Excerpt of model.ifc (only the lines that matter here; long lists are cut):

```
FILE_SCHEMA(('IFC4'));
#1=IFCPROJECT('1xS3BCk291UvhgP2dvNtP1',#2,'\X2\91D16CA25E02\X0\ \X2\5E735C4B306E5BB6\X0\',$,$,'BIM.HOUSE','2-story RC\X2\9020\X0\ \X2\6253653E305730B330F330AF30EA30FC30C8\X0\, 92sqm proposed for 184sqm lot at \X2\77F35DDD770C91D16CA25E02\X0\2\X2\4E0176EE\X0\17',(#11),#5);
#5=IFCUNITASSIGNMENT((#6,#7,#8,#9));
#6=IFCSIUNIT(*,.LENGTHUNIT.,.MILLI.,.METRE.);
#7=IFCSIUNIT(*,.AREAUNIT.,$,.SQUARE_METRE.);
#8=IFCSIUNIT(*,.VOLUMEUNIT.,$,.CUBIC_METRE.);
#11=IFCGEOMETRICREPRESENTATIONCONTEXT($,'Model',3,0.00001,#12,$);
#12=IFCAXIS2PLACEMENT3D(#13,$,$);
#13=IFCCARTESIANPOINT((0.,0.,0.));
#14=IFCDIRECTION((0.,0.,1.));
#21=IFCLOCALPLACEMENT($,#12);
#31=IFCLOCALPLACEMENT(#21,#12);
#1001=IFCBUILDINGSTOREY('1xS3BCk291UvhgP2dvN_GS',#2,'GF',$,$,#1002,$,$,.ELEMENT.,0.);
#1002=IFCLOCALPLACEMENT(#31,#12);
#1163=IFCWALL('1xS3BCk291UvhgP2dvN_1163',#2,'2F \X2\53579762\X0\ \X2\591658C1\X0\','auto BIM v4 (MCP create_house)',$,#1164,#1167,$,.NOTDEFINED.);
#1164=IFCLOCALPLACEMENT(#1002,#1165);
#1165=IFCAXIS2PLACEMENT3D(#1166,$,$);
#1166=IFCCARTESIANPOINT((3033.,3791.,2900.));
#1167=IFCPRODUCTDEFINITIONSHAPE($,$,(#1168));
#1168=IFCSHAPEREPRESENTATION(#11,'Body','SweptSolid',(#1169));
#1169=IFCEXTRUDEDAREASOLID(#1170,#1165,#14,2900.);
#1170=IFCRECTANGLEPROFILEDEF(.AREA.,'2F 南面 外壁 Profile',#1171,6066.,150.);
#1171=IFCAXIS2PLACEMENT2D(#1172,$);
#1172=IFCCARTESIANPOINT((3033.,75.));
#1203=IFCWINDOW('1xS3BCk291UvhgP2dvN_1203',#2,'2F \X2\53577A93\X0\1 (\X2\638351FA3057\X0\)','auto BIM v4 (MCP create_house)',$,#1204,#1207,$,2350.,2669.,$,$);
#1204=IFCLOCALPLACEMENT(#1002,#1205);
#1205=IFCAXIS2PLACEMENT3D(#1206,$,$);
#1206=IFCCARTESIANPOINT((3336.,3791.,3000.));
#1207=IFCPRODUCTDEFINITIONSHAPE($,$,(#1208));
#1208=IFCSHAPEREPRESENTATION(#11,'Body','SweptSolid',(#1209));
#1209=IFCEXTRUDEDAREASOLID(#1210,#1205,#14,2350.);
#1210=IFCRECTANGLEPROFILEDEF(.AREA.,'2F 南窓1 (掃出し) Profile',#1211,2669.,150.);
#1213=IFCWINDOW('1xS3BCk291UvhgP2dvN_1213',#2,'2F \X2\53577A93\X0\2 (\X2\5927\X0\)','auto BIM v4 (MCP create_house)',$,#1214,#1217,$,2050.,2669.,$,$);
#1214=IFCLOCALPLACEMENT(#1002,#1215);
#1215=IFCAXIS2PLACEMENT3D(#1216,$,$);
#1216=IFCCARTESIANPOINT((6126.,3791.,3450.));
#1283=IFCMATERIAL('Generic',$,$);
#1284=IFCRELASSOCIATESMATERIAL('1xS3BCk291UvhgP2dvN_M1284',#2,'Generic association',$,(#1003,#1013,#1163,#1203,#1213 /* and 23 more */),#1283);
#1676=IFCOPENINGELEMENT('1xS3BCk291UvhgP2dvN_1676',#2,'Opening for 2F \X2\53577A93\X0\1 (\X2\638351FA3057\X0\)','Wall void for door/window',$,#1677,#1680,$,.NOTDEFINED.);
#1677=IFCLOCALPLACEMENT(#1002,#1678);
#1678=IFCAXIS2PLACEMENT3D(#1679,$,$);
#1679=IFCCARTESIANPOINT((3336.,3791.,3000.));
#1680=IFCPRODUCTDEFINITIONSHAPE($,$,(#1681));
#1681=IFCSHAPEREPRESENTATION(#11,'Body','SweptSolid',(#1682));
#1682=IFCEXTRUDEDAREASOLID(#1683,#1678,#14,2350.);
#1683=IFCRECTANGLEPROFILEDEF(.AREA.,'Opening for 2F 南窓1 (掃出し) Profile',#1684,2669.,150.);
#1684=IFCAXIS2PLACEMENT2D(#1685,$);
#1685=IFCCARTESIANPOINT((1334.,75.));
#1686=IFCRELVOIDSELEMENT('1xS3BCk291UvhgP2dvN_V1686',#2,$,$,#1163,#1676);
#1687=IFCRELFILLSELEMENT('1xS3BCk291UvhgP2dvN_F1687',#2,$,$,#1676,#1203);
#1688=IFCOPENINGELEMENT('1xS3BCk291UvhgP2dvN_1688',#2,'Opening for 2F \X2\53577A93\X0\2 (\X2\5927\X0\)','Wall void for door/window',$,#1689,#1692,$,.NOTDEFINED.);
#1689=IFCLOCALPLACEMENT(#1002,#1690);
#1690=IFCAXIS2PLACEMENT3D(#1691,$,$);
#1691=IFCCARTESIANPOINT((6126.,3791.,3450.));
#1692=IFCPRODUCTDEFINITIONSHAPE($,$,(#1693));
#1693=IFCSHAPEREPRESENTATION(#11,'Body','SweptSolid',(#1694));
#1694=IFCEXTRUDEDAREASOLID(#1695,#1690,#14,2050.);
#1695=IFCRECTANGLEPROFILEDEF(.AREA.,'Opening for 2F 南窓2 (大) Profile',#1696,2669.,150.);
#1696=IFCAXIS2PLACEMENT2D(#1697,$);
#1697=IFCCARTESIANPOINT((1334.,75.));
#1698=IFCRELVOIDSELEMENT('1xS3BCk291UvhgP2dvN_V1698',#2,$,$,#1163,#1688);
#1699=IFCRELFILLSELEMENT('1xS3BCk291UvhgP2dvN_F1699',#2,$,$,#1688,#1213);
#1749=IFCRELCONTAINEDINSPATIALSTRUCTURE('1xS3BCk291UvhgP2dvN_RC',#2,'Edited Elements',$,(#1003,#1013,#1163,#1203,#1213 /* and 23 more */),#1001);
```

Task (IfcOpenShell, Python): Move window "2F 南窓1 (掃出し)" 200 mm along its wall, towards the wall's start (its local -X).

```python
import ifcopenshell
import ifcopenshell.api.geometry
import ifcopenshell.util.placement

model = ifcopenshell.open("model.ifc")

window = model.by_guid("1xS3BCk291UvhgP2dvN_1203")
opening = window.FillsVoids[0].RelatingOpeningElement
wall = opening.VoidsElements[0].RelatingBuildingElement

wall_matrix = ifcopenshell.util.placement.get_local_placement(wall.ObjectPlacement)
shift = wall_matrix[:3, 0] * -200.0
before = ifcopenshell.util.placement.get_local_placement(window.ObjectPlacement)[:3, 3].copy()

# The window is not placed relative to its opening, so move both.
for product in (opening, window):
    matrix = ifcopenshell.util.placement.get_local_placement(product.ObjectPlacement)
    matrix[:3, 3] += shift
    ifcopenshell.api.geometry.edit_object_placement(model, product=product, matrix=matrix, is_si=False)

after = ifcopenshell.util.placement.get_local_placement(window.ObjectPlacement)[:3, 3]
print("window moved by", (after - before).round(3) + 0.0)

model.write("model_rev.ifc")
```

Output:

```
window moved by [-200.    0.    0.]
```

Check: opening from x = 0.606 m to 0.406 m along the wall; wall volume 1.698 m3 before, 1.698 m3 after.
